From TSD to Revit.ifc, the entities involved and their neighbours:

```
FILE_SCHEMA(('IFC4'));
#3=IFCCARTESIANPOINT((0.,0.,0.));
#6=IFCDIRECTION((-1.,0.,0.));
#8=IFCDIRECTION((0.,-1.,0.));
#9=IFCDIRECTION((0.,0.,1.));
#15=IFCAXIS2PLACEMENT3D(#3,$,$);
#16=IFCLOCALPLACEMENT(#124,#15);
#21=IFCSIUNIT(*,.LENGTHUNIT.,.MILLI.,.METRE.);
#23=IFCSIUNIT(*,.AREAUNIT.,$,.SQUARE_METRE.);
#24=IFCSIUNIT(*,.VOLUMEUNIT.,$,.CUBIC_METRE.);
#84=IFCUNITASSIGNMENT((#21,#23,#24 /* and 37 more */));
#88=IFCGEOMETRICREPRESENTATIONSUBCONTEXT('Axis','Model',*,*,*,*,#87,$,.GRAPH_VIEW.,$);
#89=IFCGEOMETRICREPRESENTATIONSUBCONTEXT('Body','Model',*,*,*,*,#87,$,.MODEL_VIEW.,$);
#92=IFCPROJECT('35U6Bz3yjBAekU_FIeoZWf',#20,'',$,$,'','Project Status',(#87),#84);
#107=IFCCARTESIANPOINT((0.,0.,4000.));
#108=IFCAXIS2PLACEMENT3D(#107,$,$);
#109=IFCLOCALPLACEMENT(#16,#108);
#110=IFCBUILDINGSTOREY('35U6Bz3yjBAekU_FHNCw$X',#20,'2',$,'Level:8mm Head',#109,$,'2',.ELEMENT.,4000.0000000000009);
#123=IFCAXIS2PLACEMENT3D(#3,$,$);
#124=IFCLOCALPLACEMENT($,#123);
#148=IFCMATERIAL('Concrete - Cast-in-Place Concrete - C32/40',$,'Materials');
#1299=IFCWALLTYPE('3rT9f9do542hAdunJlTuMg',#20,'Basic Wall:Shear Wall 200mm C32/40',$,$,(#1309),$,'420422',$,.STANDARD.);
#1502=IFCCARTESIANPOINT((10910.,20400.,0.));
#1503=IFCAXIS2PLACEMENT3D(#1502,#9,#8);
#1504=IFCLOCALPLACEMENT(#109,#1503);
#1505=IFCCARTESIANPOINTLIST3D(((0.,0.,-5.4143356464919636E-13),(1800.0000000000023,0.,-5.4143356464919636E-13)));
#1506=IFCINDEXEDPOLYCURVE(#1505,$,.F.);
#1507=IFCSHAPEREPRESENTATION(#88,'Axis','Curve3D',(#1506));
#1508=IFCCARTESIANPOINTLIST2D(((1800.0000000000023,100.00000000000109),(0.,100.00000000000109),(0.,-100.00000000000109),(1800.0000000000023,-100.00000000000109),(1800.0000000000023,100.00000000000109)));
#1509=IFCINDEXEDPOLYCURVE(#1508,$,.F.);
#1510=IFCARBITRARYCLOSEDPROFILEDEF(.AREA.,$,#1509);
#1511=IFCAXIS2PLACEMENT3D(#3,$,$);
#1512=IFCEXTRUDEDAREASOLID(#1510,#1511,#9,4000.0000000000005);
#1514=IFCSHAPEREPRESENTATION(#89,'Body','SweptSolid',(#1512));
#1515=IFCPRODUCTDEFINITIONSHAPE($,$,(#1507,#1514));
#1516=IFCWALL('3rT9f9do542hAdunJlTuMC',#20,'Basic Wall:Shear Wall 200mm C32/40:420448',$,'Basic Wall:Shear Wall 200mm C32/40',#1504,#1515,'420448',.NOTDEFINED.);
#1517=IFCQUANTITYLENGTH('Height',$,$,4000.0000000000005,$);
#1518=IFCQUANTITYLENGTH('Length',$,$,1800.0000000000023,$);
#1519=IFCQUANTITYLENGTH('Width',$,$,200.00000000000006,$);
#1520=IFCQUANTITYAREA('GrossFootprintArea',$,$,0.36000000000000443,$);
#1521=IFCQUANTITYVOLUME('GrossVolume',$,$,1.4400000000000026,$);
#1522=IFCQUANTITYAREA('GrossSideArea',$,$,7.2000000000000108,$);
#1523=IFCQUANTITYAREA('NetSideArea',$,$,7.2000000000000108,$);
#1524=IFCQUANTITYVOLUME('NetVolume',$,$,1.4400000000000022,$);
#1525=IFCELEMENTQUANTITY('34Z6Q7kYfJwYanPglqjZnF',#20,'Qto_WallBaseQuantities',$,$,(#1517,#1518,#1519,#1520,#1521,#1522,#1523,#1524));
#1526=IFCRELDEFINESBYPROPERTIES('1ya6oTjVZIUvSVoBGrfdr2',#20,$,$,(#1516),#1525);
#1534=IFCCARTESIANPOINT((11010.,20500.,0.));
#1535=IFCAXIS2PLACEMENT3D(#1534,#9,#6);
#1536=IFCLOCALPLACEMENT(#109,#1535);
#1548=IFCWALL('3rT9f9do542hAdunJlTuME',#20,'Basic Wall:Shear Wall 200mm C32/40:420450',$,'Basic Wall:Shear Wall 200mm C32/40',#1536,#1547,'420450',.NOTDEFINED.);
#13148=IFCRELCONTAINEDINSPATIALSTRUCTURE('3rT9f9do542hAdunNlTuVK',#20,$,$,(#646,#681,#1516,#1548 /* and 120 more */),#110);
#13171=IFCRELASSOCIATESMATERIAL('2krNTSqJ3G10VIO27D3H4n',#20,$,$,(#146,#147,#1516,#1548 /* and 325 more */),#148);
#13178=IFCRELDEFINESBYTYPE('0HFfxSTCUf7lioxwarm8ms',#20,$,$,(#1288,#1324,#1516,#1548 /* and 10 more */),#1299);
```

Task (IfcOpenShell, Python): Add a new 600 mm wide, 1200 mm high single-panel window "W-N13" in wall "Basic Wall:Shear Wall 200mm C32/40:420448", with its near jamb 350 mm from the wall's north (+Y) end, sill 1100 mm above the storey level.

```python
import numpy as np
import ifcopenshell
import ifcopenshell.api.feature
import ifcopenshell.api.geometry
import ifcopenshell.api.pset
import ifcopenshell.api.root
import ifcopenshell.api.spatial
import ifcopenshell.geom
import ifcopenshell.util.element
import ifcopenshell.util.placement
import ifcopenshell.util.representation
import ifcopenshell.util.shape
import ifcopenshell.util.unit

model = ifcopenshell.open("TSD to Revit.ifc")
unit_scale = ifcopenshell.util.unit.calculate_unit_scale(model)
area_scale = ifcopenshell.util.unit.calculate_unit_scale(model, "AREAUNIT")
volume_scale = ifcopenshell.util.unit.calculate_unit_scale(model, "VOLUMEUNIT")
settings = ifcopenshell.geom.settings()


def volume(element):
    """Net volume in cubic metres, openings subtracted."""
    shape = ifcopenshell.geom.create_shape(settings, element)
    return ifcopenshell.util.shape.get_volume(shape.geometry)


wall = model.by_guid("3rT9f9do542hAdunJlTuMC")
storey = ifcopenshell.util.element.get_container(wall, ifc_class="IfcBuildingStorey")
context = ifcopenshell.util.representation.get_context(model, "Model", "Body", "MODEL_VIEW")
before = volume(wall)

width, height, from_end, sill = 0.6, 1.2, 0.35, 1.1  # metres

# The wall runs along its own X axis, and the end named is its -X end.
wall_shape = ifcopenshell.geom.create_shape(settings, wall)
x, y, z = ifcopenshell.util.shape.get_vertices(wall_shape.geometry).T
start = x.min() + from_end
face, thickness = float(y.min()), float(y.max() - y.min())
wall_matrix = ifcopenshell.util.placement.get_local_placement(wall.ObjectPlacement)
level = ifcopenshell.util.placement.get_local_placement(storey.ObjectPlacement)[2, 3]


def in_wall(x, y):
    """Placement at x, y metres in the wall's axes, at sill height."""
    matrix = wall_matrix.copy()
    matrix[:, 3] = wall_matrix @ np.array([x / unit_scale, y / unit_scale, 0.0, 1.0])
    matrix[2, 3] = level + sill / unit_scale
    return matrix


# Opening: a box that overshoots both wall faces by 50 mm.
opening = ifcopenshell.api.root.create_entity(model, ifc_class="IfcOpeningElement", predefined_type="OPENING")
box = ifcopenshell.api.geometry.add_wall_representation(
    model, context=context, length=width, height=height, thickness=thickness + 0.1
)
ifcopenshell.api.geometry.assign_representation(model, product=opening, representation=box)
ifcopenshell.api.geometry.edit_object_placement(model, product=opening, matrix=in_wall(start, face - 0.05), is_si=False)
ifcopenshell.api.feature.add_feature(model, feature=opening, element=wall)

window = ifcopenshell.api.root.create_entity(model, ifc_class="IfcWindow", name="W-N13", predefined_type="WINDOW")
window.OverallWidth, window.OverallHeight = width / unit_scale, height / unit_scale
window.PartitioningType = "SINGLE_PANEL"
body = ifcopenshell.api.geometry.add_window_representation(
    model,
    context=context,
    overall_width=window.OverallWidth,
    overall_height=window.OverallHeight,
    partition_type="SINGLE_PANEL",
)
ifcopenshell.api.geometry.assign_representation(model, product=window, representation=body)
ifcopenshell.api.spatial.assign_container(model, products=[window], relating_structure=storey)
ifcopenshell.api.feature.add_filling(model, opening=opening, element=window)

# Centre the window in the wall's thickness.
ifcopenshell.api.geometry.edit_object_placement(model, product=window, matrix=in_wall(start, face), is_si=False)
window_shape = ifcopenshell.geom.create_shape(settings, window)
depth = ifcopenshell.util.shape.get_vertices(window_shape.geometry)[:, 1]
offset = face + thickness / 2 - (depth.min() + depth.max()) / 2
ifcopenshell.api.geometry.edit_object_placement(model, product=window, matrix=in_wall(start, offset), is_si=False)

after = volume(wall)

# Update the wall's stored quantities.
qto = model.by_id(ifcopenshell.util.element.get_pset(wall, "Qto_WallBaseQuantities", should_inherit=False)["id"])
ifcopenshell.api.pset.edit_qto(model, qto=qto, properties={
    "NetSideArea": after / thickness / area_scale,
    "NetVolume": after / volume_scale,
})

print(f"wall volume {before:.3f} -> {after:.3f} m3")

model.write("TSD to Revit_rev.ifc")
```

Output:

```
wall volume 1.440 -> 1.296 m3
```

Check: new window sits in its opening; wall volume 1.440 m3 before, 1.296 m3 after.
